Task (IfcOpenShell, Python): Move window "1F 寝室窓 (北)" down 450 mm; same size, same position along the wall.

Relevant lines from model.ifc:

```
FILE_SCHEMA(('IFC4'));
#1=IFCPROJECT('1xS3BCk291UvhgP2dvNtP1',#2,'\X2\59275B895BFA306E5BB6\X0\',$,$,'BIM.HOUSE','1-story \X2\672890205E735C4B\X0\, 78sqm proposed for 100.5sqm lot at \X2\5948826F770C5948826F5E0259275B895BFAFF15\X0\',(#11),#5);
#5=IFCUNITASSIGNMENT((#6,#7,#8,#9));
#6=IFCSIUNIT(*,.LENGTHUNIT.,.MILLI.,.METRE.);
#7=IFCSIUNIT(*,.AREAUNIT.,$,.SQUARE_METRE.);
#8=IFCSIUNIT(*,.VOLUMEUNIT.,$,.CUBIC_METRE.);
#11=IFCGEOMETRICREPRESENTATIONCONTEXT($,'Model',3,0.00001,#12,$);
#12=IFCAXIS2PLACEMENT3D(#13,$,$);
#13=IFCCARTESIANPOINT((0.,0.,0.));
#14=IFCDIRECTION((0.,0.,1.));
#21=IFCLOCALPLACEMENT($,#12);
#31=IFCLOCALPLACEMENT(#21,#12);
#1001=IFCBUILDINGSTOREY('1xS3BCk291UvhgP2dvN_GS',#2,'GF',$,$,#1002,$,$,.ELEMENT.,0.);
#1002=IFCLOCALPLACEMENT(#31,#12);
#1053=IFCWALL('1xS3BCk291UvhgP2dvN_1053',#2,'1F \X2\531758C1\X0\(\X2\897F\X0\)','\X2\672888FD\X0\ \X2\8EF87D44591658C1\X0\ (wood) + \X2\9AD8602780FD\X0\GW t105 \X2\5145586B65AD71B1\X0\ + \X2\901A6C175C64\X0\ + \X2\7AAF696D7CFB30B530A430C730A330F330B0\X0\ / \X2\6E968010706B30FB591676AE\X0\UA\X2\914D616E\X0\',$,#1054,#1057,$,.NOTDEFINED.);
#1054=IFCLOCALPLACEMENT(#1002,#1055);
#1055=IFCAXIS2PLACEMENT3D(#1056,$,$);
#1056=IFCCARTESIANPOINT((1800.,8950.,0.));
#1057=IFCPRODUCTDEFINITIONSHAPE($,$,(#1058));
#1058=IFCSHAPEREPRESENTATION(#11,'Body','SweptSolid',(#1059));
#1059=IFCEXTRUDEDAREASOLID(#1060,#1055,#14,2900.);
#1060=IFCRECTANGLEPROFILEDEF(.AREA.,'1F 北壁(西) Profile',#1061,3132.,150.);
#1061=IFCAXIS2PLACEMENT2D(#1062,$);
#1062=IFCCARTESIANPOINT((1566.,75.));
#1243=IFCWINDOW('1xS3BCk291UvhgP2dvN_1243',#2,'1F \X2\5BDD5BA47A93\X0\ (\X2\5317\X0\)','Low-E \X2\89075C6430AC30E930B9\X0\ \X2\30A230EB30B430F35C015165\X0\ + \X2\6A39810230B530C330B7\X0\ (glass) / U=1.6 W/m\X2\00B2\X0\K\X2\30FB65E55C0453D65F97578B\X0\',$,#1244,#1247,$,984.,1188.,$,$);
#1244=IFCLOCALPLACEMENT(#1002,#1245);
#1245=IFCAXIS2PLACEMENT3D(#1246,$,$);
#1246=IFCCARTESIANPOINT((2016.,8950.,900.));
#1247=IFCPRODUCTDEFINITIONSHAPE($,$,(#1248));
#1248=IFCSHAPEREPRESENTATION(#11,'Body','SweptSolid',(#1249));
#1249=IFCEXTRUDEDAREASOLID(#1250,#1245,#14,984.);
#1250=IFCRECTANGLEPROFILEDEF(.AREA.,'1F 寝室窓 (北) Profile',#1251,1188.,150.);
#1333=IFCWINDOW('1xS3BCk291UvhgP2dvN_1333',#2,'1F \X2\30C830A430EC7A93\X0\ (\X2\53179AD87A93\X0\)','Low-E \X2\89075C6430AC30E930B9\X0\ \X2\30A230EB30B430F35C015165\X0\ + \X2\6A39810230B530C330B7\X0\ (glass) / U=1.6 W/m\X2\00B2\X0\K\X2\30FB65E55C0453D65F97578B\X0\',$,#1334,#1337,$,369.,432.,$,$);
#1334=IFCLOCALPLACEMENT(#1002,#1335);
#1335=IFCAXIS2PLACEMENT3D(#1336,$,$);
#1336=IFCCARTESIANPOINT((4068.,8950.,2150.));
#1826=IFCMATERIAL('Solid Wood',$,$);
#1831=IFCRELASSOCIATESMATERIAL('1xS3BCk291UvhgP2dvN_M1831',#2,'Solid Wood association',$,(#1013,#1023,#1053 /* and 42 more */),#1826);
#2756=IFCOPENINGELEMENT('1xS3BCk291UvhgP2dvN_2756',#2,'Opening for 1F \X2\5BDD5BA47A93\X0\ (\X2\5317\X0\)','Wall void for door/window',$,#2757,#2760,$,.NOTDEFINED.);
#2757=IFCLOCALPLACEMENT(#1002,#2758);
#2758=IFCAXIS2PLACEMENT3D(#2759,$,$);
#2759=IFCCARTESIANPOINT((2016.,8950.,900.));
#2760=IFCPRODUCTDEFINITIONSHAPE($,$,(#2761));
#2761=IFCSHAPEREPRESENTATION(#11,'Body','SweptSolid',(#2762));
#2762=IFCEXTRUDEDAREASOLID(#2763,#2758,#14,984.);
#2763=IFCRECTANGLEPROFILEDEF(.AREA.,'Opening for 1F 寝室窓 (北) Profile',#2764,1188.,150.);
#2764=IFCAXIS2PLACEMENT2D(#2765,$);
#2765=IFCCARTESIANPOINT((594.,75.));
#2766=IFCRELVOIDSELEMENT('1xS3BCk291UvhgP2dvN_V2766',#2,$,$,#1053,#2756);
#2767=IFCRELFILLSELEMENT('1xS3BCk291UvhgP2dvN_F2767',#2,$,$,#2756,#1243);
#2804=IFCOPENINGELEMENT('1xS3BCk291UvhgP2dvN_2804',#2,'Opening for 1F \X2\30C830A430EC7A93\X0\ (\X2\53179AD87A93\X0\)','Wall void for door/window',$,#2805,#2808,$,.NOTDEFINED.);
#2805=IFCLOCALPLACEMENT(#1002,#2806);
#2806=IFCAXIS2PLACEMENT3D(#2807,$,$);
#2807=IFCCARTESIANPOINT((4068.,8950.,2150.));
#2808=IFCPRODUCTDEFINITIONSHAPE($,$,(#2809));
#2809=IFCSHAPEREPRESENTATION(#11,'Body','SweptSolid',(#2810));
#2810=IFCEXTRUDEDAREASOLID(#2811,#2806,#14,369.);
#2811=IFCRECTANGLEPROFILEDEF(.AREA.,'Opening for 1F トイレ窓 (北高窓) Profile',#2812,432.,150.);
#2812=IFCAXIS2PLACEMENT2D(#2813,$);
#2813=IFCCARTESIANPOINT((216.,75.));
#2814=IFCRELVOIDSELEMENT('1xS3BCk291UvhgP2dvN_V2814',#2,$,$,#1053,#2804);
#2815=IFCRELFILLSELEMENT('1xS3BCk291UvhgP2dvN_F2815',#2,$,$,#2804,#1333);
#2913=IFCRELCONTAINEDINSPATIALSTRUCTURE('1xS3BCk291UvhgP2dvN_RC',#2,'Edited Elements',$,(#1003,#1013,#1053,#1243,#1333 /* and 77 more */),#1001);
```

```python
import numpy as np
import ifcopenshell
import ifcopenshell.api.geometry
import ifcopenshell.util.placement
import ifcopenshell.util.unit

model = ifcopenshell.open("model.ifc")
unit_scale = ifcopenshell.util.unit.calculate_unit_scale(model)

window = model.by_guid("1xS3BCk291UvhgP2dvN_1243")
opening = window.FillsVoids[0].RelatingOpeningElement
dz = -0.45 / unit_scale

shift = np.array([0.0, 0.0, dz])
# The window is not placed relative to its opening, so move both.
for product in (opening, window):
    matrix = ifcopenshell.util.placement.get_local_placement(product.ObjectPlacement)
    matrix[:3, 3] += shift
    ifcopenshell.api.geometry.edit_object_placement(model, product=product, matrix=matrix, is_si=False)

print(f"moved by {dz * unit_scale:+.3f} m")

model.write("model_updated.ifc")
```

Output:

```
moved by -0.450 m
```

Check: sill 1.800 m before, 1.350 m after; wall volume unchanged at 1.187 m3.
